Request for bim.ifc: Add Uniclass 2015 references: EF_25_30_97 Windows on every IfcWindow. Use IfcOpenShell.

First a look at what the model holds.

```python
import ifcopenshell

model = ifcopenshell.open("bim.ifc")
print(model.schema)
print("classifications:", [c.Name for c in model.by_type("IfcClassification")])
for ifc_class in ("IfcDoor", "IfcRoof", "IfcStair", "IfcWall", "IfcWindow"):
    print(ifc_class, len(model.by_type(ifc_class)))
```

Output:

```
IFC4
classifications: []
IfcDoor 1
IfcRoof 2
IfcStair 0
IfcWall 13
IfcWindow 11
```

```python
import ifcopenshell
import ifcopenshell.api.classification

model = ifcopenshell.open("bim.ifc")

system = ifcopenshell.api.classification.add_classification(model, classification="Uniclass 2015")

codes = {
    "IfcWindow": ("EF_25_30_97", "Windows"),
}
for ifc_class, (code, name) in codes.items():
    products = model.by_type(ifc_class)
    ifcopenshell.api.classification.add_reference(
        model, products=products, classification=system, identification=code, name=name
    )
    print(code, len(products))

model.write("bim_updated.ifc")
```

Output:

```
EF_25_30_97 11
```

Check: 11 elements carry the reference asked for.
